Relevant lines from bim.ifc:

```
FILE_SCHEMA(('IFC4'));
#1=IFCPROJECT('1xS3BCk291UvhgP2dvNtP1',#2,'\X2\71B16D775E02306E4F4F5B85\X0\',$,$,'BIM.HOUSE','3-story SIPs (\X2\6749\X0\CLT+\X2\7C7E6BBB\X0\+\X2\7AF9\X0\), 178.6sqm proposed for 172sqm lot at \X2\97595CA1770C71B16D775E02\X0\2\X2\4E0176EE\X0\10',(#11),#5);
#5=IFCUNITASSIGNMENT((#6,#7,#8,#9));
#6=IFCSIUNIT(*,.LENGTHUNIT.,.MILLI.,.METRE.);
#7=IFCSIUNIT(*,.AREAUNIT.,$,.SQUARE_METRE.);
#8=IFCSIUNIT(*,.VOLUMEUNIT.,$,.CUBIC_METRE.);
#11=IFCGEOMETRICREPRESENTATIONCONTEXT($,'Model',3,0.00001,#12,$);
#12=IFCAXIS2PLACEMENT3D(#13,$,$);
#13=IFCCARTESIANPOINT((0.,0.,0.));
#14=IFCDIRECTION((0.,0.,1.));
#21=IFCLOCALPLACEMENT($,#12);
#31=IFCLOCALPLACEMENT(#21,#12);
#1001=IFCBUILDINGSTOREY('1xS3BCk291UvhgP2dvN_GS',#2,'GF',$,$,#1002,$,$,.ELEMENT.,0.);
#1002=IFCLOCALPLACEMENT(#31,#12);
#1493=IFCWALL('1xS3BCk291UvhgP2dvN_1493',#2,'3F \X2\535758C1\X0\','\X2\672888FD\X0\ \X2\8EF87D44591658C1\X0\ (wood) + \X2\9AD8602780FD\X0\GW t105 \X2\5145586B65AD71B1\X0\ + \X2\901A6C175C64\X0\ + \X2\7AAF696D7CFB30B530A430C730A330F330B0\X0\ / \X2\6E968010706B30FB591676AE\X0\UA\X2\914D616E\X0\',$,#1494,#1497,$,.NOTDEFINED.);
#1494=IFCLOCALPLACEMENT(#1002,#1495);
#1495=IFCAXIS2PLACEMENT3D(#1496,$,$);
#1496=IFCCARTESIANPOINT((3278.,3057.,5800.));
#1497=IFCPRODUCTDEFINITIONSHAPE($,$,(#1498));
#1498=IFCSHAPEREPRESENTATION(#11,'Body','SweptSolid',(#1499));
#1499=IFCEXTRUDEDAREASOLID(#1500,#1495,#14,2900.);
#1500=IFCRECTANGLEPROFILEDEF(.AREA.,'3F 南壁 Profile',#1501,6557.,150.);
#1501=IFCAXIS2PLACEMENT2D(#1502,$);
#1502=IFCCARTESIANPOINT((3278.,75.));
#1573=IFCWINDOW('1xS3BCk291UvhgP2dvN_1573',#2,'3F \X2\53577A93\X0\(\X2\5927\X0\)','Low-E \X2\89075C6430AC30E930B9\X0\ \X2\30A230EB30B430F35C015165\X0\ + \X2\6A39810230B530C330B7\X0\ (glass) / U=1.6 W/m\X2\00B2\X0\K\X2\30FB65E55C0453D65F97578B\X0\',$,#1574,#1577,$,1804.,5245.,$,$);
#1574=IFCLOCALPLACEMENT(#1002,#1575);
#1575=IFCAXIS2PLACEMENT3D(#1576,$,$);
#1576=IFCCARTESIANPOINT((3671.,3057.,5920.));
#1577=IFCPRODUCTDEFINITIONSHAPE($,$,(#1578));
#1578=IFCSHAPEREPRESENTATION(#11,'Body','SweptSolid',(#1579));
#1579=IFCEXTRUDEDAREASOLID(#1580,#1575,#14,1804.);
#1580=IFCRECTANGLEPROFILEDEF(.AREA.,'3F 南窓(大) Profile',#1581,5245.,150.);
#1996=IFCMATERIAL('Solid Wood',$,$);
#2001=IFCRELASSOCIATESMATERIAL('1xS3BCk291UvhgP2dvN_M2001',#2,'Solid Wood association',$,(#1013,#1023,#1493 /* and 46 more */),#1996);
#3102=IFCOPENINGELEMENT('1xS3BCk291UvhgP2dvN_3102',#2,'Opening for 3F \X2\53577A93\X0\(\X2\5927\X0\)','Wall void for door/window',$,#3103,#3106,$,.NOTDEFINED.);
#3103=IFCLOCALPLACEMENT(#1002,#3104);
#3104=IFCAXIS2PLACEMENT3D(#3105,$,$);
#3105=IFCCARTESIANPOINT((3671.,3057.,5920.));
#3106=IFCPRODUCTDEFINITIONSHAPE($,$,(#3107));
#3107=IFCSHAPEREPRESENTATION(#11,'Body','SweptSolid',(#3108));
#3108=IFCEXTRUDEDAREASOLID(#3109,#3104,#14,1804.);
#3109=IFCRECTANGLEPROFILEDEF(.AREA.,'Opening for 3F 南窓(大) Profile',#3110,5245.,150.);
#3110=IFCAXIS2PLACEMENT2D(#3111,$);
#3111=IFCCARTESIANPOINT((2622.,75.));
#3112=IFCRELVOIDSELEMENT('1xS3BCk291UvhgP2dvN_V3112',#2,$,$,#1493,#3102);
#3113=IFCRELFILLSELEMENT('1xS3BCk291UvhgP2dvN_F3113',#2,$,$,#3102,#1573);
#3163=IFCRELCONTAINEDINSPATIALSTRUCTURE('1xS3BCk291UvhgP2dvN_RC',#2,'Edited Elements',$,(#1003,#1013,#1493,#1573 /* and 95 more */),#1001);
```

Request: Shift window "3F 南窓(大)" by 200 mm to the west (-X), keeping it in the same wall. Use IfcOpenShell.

```python
import ifcopenshell
import ifcopenshell.api.geometry
import ifcopenshell.util.placement

model = ifcopenshell.open("bim.ifc")

window = model.by_guid("1xS3BCk291UvhgP2dvN_1573")
opening = window.FillsVoids[0].RelatingOpeningElement
wall = opening.VoidsElements[0].RelatingBuildingElement

wall_matrix = ifcopenshell.util.placement.get_local_placement(wall.ObjectPlacement)
shift = wall_matrix[:3, 0] * -200.0
before = ifcopenshell.util.placement.get_local_placement(window.ObjectPlacement)[:3, 3].copy()

# The window is not placed relative to its opening, so move both.
for product in (opening, window):
    matrix = ifcopenshell.util.placement.get_local_placement(product.ObjectPlacement)
    matrix[:3, 3] += shift
    ifcopenshell.api.geometry.edit_object_placement(model, product=product, matrix=matrix, is_si=False)

after = ifcopenshell.util.placement.get_local_placement(window.ObjectPlacement)[:3, 3]
print("window moved by", (after - before).round(3) + 0.0)

model.write("bim_edited.ifc")
```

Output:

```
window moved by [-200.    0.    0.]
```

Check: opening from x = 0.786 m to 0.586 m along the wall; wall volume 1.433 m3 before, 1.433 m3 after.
